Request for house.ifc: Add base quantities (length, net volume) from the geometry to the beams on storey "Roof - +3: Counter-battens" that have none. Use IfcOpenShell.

First a look at what the model holds.

```python
import ifcopenshell
import ifcopenshell.util.element
import ifcopenshell.util.unit

model = ifcopenshell.open("house.ifc")
print(model.schema)
for unit_type in ("LENGTHUNIT", "AREAUNIT", "VOLUMEUNIT"):
    print(unit_type, ifcopenshell.util.unit.calculate_unit_scale(model, unit_type))
storey = next(s for s in model.by_type("IfcBuildingStorey") if s.Name == "Roof - +3: Counter-battens")
beams = [e for e in ifcopenshell.util.element.get_decomposition(storey) if e.is_a("IfcBeam")]
for e in sorted(beams, key=lambda e: e.id()):
    print(e.id(), e.is_a(), e.Name, list(ifcopenshell.util.element.get_psets(e, qtos_only=True)), sep=" | ")
```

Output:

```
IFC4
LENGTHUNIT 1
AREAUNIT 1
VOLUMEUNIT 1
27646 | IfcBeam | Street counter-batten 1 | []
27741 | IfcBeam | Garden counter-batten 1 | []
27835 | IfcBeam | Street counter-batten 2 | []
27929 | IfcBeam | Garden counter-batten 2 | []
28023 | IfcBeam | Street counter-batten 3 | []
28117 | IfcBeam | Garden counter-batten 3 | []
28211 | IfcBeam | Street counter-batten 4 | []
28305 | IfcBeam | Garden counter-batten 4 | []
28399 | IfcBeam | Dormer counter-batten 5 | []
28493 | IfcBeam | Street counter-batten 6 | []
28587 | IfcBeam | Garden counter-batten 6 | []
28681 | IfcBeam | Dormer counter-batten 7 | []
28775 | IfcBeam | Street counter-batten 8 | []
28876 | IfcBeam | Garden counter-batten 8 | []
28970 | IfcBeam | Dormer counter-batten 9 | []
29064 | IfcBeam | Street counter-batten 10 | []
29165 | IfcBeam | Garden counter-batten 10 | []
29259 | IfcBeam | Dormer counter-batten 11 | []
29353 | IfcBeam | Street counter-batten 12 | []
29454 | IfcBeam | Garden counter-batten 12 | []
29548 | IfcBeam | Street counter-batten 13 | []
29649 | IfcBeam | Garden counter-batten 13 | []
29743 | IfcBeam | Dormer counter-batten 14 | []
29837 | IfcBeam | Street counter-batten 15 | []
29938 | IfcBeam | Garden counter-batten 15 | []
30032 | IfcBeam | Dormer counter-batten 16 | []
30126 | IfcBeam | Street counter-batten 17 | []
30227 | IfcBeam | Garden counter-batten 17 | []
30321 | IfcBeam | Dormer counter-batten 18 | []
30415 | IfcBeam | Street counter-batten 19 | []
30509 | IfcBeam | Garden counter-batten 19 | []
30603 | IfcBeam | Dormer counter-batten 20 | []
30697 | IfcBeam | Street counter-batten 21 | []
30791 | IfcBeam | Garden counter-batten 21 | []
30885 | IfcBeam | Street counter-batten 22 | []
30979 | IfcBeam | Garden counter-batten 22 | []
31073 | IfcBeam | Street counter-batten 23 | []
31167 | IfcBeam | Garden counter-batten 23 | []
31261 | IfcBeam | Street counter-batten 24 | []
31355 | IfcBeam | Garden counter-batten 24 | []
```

```python
import ifcopenshell
import ifcopenshell.api.pset
import ifcopenshell.geom
import ifcopenshell.util.element
import ifcopenshell.util.shape
import ifcopenshell.util.unit

model = ifcopenshell.open("house.ifc")
unit_scale = ifcopenshell.util.unit.calculate_unit_scale(model)
volume_scale = ifcopenshell.util.unit.calculate_unit_scale(model, "VOLUMEUNIT")
settings = ifcopenshell.geom.settings()

storey = next(s for s in model.by_type("IfcBuildingStorey") if s.Name == "Roof - +3: Counter-battens")
beams = [e for e in ifcopenshell.util.element.get_decomposition(storey) if e.is_a("IfcBeam")]

for e in sorted(beams, key=lambda e: e.id()):
    if ifcopenshell.util.element.get_psets(e, qtos_only=True, should_inherit=False):
        continue
    # Geometry comes back in metres, in the element's own axes.
    shape = ifcopenshell.geom.create_shape(settings, e)
    values = {
        "Length": ifcopenshell.util.shape.get_max_xyz(shape.geometry) / unit_scale,
        "NetVolume": ifcopenshell.util.shape.get_volume(shape.geometry) / volume_scale,
    }
    qto = ifcopenshell.api.pset.add_qto(model, product=e, name="Qto_BeamBaseQuantities")
    ifcopenshell.api.pset.edit_qto(model, qto=qto, properties=values)
    print(e.id(), {k: round(v, 3) for k, v in values.items()})

model.write("house_edited.ifc")
```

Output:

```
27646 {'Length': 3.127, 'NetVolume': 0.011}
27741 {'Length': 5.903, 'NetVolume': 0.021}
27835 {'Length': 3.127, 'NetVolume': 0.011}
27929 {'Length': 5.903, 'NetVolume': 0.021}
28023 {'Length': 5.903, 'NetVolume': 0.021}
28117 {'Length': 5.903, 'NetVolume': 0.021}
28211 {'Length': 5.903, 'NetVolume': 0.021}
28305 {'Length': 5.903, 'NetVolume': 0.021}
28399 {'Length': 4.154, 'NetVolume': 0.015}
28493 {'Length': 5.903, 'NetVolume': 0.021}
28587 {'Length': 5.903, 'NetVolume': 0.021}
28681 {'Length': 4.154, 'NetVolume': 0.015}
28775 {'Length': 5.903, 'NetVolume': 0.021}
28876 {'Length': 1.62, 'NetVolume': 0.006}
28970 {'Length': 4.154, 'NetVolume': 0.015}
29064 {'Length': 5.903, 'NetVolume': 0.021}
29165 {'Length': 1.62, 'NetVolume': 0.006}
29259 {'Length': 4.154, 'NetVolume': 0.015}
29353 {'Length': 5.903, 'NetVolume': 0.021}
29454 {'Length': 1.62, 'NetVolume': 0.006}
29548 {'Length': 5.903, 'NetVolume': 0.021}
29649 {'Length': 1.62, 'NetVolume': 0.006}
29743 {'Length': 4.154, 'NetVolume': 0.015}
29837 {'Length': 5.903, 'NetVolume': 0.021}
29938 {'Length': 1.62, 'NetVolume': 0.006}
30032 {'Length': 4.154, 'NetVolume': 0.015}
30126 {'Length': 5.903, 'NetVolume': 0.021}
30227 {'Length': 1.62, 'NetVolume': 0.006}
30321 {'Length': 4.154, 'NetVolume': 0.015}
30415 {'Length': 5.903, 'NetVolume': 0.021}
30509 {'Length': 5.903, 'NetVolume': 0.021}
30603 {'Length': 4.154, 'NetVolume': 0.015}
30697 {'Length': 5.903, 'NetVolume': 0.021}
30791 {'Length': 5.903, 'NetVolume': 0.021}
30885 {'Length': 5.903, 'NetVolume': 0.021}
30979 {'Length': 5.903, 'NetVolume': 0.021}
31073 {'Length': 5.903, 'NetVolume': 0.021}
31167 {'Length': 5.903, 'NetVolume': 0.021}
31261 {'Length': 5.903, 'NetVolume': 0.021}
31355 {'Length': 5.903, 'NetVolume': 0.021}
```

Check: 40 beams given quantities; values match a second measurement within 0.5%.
